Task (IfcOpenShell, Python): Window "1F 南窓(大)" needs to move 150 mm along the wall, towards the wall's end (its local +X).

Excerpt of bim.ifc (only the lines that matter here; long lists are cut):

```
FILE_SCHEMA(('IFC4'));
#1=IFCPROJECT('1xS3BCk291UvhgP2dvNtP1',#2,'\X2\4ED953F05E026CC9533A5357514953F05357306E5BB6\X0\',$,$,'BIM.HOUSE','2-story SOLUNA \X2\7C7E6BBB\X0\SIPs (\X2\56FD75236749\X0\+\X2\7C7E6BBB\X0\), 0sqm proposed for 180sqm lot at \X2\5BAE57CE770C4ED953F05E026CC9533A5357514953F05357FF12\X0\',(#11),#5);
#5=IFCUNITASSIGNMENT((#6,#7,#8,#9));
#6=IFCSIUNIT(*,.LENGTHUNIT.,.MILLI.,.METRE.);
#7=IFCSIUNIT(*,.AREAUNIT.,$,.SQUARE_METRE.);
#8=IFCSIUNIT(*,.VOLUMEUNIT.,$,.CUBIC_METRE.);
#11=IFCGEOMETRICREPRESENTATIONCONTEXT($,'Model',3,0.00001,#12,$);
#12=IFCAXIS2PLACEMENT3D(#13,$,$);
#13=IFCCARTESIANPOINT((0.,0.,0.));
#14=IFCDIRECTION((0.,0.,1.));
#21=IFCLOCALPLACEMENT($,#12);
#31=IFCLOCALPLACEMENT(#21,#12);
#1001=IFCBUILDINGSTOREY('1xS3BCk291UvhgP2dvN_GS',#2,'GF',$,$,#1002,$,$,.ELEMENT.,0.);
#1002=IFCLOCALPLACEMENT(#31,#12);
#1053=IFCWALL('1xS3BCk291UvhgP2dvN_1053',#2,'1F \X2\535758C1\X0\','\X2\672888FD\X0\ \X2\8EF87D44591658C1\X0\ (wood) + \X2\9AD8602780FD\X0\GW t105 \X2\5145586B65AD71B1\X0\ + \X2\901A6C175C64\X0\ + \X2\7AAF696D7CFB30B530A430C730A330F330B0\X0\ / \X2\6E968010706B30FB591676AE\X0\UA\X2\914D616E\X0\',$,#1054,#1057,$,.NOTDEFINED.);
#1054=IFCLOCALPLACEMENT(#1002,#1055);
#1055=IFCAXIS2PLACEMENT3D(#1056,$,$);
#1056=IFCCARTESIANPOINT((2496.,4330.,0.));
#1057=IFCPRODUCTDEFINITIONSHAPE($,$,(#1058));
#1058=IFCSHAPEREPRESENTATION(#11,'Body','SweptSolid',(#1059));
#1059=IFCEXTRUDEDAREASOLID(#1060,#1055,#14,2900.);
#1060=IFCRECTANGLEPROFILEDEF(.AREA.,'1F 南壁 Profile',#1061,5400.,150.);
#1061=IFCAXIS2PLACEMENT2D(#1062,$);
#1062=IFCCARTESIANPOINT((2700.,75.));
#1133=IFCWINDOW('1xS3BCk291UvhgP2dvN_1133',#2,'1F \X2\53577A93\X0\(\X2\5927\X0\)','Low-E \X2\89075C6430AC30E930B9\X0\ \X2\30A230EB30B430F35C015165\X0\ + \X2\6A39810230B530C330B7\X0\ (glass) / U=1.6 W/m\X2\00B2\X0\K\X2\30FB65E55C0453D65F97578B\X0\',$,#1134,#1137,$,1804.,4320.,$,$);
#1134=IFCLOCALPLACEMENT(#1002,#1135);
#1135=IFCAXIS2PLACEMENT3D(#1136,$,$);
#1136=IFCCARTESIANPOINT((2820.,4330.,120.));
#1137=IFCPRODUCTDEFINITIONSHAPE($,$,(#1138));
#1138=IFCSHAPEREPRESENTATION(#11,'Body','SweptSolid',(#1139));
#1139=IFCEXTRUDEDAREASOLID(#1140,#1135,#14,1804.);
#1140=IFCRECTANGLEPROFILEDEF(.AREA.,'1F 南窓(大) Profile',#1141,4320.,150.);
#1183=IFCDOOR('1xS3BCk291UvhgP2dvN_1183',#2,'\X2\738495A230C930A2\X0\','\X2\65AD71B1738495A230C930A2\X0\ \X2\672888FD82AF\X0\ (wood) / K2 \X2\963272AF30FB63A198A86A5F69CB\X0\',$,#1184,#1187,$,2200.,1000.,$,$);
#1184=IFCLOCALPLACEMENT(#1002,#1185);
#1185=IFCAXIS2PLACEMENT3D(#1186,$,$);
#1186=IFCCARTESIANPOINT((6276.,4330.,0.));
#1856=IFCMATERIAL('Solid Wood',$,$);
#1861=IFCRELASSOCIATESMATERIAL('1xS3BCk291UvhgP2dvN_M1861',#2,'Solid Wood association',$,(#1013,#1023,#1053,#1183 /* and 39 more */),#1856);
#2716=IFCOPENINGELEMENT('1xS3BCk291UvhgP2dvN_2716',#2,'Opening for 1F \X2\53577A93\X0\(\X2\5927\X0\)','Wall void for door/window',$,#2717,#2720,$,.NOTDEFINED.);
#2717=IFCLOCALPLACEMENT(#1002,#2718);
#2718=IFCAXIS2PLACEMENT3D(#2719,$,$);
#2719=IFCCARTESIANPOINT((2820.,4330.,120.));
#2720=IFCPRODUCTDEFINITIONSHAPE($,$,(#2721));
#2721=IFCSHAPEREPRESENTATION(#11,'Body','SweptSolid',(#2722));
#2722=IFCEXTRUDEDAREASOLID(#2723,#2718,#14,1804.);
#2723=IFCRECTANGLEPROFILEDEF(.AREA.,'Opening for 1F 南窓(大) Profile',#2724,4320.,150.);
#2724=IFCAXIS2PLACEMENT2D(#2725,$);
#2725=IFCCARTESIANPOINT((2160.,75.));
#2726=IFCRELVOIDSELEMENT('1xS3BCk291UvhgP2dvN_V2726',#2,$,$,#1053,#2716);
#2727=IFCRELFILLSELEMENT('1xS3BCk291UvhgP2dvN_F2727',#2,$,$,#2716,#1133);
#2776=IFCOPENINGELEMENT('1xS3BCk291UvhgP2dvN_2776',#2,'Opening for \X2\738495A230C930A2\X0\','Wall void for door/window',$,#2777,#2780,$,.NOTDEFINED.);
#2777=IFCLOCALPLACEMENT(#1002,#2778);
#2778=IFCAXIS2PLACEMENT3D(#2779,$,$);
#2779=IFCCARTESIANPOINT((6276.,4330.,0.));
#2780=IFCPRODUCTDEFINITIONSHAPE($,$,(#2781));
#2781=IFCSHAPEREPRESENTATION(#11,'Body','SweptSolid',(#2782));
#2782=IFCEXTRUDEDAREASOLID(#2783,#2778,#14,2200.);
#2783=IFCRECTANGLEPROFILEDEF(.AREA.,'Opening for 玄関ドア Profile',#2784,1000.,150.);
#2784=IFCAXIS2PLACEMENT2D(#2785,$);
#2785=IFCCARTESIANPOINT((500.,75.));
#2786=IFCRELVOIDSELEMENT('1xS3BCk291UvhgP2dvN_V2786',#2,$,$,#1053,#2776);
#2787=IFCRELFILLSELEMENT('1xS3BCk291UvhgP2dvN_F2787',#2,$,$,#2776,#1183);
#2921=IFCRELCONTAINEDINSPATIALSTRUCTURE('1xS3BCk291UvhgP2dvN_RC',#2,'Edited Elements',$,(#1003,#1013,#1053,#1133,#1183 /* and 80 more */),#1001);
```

```python
import ifcopenshell
import ifcopenshell.api.geometry
import ifcopenshell.util.placement
import ifcopenshell.util.unit

model = ifcopenshell.open("bim.ifc")
unit_scale = ifcopenshell.util.unit.calculate_unit_scale(model)

window = model.by_guid("1xS3BCk291UvhgP2dvN_1133")
opening = window.FillsVoids[0].RelatingOpeningElement
wall = opening.VoidsElements[0].RelatingBuildingElement

wall_matrix = ifcopenshell.util.placement.get_local_placement(wall.ObjectPlacement)
shift = wall_matrix[:3, 0] * 0.15 / unit_scale
before = ifcopenshell.util.placement.get_local_placement(window.ObjectPlacement)[:3, 3].copy()

# The window is not placed relative to its opening, so move both.
for product in (opening, window):
    matrix = ifcopenshell.util.placement.get_local_placement(product.ObjectPlacement)
    matrix[:3, 3] += shift
    ifcopenshell.api.geometry.edit_object_placement(model, product=product, matrix=matrix, is_si=False)

after = ifcopenshell.util.placement.get_local_placement(window.ObjectPlacement)[:3, 3]
print("window moved by", (after - before).round(3) + 0.0)

model.write("bim-out.ifc")
```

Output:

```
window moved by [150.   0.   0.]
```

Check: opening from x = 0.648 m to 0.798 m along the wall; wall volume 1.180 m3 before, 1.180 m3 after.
